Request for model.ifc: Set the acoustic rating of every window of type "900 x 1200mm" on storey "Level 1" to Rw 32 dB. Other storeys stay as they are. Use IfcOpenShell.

First a look at what the model holds.

```python
import ifcopenshell
import ifcopenshell.util.element

model = ifcopenshell.open("model.ifc")
print(model.schema)
storey = next(s for s in model.by_type("IfcBuildingStorey") if s.Name == "Level 1")
windows = [e for e in ifcopenshell.util.element.get_decomposition(storey) if e.is_a("IfcWindow")]
seen = {}
for e in windows:
    element_type = ifcopenshell.util.element.get_type(e)
    key = (element_type.Name if element_type != e and element_type else None, ifcopenshell.util.element.get_pset(e, "Pset_WindowCommon", "AcousticRating"))
    seen[key] = seen.get(key, 0) + 1
for (name, value), count in sorted(seen.items(), key=str):
    print(count, "x", name, "|", value)
```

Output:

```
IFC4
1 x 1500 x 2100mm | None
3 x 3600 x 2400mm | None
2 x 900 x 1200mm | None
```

```python
import ifcopenshell
import ifcopenshell.api.pset
import ifcopenshell.util.element

model = ifcopenshell.open("model.ifc")

storey = next(s for s in model.by_type("IfcBuildingStorey") if s.Name == "Level 1")
windows = [e for e in ifcopenshell.util.element.get_decomposition(storey) if e.is_a("IfcWindow")]

count = 0
for e in windows:
    element_type = ifcopenshell.util.element.get_type(e)
    if element_type in (None, e) or element_type.Name != "900 x 1200mm":
        continue
    # add_pset returns the element's existing set when there is one.
    pset = ifcopenshell.api.pset.add_pset(model, product=e, name="Pset_WindowCommon")
    ifcopenshell.api.pset.edit_pset(model, pset=pset, properties={"AcousticRating": "Rw 32 dB"})
    count += 1

print(count, "windows updated")

model.write("model_edited.ifc")
```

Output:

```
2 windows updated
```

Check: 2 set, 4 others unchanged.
